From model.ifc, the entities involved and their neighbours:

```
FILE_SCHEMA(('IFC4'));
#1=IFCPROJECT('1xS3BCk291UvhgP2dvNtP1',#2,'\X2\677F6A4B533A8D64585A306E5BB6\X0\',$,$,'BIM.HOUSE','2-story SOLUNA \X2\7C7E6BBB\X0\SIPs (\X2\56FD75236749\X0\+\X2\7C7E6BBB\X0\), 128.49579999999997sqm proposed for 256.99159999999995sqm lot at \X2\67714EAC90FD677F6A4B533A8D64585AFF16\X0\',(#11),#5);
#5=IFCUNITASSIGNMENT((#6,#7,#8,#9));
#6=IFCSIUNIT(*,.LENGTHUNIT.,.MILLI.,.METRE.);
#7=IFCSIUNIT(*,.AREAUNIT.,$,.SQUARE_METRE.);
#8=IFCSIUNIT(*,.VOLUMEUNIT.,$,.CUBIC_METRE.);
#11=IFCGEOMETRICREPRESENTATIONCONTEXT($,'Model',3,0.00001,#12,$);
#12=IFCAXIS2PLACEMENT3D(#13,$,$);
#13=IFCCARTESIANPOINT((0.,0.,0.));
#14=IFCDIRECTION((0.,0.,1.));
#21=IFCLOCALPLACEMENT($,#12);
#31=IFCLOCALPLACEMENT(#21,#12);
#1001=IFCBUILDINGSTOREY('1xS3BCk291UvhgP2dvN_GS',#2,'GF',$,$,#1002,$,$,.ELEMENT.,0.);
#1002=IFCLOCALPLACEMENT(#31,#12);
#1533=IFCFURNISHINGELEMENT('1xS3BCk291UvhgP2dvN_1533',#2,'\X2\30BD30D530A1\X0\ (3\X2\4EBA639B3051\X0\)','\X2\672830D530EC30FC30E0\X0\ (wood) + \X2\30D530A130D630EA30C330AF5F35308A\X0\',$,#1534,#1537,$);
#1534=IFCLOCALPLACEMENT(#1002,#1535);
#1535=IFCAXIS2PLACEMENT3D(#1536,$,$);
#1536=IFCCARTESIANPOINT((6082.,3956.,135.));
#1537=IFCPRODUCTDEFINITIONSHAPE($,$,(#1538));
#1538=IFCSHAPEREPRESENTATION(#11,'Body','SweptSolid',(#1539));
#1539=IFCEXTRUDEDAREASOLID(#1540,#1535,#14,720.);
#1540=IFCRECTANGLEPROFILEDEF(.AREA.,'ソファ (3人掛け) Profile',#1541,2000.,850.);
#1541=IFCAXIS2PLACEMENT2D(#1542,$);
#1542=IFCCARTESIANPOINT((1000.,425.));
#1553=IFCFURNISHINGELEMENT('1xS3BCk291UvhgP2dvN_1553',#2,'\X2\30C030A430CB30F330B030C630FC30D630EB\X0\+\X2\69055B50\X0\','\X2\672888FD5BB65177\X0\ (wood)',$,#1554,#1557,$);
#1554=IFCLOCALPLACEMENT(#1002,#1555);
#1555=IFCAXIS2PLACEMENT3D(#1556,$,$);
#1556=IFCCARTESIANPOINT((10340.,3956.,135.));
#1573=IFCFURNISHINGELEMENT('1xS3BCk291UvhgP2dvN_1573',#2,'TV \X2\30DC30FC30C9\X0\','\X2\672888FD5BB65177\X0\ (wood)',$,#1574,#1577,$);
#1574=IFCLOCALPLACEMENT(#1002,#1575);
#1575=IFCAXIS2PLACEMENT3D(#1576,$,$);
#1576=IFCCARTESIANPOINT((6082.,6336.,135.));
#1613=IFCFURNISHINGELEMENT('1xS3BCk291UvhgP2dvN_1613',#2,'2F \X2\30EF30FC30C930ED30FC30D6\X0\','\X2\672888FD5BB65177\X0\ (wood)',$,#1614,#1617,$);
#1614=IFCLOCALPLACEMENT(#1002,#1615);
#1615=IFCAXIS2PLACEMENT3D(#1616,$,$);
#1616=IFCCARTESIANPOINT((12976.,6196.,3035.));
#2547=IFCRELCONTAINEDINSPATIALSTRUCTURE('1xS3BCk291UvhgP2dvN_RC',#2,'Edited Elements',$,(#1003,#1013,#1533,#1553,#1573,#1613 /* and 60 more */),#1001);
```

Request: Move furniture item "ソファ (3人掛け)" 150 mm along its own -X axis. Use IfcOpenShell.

```python
import ifcopenshell
import ifcopenshell.api.geometry
import ifcopenshell.util.placement

model = ifcopenshell.open("model.ifc")

item = model.by_id(1533)
matrix = ifcopenshell.util.placement.get_local_placement(item.ObjectPlacement)
matrix[:3, 3] -= matrix[:3, 0] * 150.0
ifcopenshell.api.geometry.edit_object_placement(model, product=item, matrix=matrix, is_si=False)

print(ifcopenshell.util.placement.get_local_placement(item.ObjectPlacement).round(3) + 0.0)

model.write("model_v2.ifc")
```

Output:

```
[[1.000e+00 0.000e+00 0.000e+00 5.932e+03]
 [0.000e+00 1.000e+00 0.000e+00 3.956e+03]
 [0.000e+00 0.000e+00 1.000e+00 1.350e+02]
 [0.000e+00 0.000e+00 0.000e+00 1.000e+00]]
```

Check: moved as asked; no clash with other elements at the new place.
